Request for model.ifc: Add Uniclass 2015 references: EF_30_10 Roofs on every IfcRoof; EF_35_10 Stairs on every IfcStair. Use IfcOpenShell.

First a look at what the model holds.

```python
import ifcopenshell

model = ifcopenshell.open("model.ifc")
print(model.schema)
print("classifications:", [c.Name for c in model.by_type("IfcClassification")])
for ifc_class in ("IfcDoor", "IfcRoof", "IfcStair", "IfcWall", "IfcWindow"):
    print(ifc_class, len(model.by_type(ifc_class)))
```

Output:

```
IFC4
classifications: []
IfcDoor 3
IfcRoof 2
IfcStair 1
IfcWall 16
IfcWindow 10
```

```python
import ifcopenshell
import ifcopenshell.api.classification

model = ifcopenshell.open("model.ifc")

system = ifcopenshell.api.classification.add_classification(model, classification="Uniclass 2015")

codes = {
    "IfcRoof": ("EF_30_10", "Roofs"),
    "IfcStair": ("EF_35_10", "Stairs"),
}
for ifc_class, (code, name) in codes.items():
    products = model.by_type(ifc_class)
    ifcopenshell.api.classification.add_reference(
        model, products=products, classification=system, identification=code, name=name
    )
    print(code, len(products))

model.write("model_rev.ifc")
```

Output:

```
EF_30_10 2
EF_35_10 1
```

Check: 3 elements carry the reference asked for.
